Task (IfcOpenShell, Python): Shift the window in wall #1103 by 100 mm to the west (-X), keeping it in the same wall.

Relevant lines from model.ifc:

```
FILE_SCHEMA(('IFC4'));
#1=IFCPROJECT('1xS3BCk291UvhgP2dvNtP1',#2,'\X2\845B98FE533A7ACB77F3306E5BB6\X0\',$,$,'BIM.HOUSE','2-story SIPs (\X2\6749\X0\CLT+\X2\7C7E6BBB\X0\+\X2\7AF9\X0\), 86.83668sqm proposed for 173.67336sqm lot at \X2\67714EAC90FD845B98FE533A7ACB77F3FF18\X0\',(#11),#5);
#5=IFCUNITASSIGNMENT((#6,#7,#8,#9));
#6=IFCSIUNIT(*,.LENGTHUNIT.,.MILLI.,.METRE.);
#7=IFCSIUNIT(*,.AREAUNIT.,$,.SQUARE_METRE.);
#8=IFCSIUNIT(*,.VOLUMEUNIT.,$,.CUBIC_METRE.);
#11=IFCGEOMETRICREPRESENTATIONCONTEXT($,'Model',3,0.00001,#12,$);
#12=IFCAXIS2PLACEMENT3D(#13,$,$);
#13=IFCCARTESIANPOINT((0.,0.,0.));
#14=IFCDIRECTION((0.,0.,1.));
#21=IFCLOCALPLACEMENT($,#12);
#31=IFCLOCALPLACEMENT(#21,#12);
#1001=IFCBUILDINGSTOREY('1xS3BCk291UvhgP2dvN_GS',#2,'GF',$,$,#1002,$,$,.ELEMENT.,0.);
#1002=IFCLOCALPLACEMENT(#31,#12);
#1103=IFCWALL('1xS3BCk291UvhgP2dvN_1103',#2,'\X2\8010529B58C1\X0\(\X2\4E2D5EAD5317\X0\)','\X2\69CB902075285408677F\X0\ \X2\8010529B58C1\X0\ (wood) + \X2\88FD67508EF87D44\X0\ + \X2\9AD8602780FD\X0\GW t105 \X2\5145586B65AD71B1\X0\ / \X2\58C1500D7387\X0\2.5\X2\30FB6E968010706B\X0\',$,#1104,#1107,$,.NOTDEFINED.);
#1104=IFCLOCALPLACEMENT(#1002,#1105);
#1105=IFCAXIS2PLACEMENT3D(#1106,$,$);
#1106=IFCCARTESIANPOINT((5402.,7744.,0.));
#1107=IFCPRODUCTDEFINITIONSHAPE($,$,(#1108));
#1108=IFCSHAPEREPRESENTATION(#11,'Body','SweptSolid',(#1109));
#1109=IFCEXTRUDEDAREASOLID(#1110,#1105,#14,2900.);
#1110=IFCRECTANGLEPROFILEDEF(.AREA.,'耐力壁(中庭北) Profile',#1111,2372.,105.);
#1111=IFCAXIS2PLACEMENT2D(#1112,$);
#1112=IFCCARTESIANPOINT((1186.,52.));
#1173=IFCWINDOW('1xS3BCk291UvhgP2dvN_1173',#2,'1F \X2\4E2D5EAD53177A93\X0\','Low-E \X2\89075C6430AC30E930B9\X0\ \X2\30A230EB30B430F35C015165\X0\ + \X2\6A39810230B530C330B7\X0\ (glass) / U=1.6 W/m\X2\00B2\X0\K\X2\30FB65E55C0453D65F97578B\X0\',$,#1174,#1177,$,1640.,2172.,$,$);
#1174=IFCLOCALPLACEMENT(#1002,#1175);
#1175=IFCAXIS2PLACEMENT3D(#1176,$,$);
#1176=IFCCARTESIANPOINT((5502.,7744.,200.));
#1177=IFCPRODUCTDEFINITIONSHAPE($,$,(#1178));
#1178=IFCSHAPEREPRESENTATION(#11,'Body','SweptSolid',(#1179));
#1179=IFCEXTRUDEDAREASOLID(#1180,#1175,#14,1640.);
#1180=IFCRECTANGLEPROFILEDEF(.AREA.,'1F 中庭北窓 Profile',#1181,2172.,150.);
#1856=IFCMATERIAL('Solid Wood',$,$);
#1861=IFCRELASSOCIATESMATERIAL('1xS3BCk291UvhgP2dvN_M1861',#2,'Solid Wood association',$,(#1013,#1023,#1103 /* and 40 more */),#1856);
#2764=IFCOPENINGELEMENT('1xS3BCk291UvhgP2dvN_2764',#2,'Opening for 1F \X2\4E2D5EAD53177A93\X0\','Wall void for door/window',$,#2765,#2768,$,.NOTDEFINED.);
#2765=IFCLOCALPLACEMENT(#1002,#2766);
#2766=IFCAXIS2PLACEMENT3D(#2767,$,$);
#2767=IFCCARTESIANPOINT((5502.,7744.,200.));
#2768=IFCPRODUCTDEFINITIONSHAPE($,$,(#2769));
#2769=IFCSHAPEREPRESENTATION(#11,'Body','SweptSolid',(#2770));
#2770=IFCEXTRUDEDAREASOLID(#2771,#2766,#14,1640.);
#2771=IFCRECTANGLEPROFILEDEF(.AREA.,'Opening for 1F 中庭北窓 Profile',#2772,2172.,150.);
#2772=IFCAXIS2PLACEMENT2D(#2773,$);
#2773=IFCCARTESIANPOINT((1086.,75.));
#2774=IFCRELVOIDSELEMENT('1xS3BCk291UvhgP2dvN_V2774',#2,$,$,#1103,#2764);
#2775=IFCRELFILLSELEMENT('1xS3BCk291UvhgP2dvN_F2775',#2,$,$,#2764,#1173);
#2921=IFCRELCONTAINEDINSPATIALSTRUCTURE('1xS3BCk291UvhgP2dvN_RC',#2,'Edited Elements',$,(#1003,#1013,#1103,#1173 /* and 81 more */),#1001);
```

```python
import ifcopenshell
import ifcopenshell.api.geometry
import ifcopenshell.util.placement
import ifcopenshell.util.unit

model = ifcopenshell.open("model.ifc")
unit_scale = ifcopenshell.util.unit.calculate_unit_scale(model)

window = model.by_id(1173)
opening = window.FillsVoids[0].RelatingOpeningElement
wall = opening.VoidsElements[0].RelatingBuildingElement

wall_matrix = ifcopenshell.util.placement.get_local_placement(wall.ObjectPlacement)
shift = wall_matrix[:3, 0] * -0.1 / unit_scale
before = ifcopenshell.util.placement.get_local_placement(window.ObjectPlacement)[:3, 3].copy()

# The window is not placed relative to its opening, so move both.
for product in (opening, window):
    matrix = ifcopenshell.util.placement.get_local_placement(product.ObjectPlacement)
    matrix[:3, 3] += shift
    ifcopenshell.api.geometry.edit_object_placement(model, product=product, matrix=matrix, is_si=False)

after = ifcopenshell.util.placement.get_local_placement(window.ObjectPlacement)[:3, 3]
print("window moved by", (after - before).round(3) + 0.0)

model.write("model-out.ifc")
```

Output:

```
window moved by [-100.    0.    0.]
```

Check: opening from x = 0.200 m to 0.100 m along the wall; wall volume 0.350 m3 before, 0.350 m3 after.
